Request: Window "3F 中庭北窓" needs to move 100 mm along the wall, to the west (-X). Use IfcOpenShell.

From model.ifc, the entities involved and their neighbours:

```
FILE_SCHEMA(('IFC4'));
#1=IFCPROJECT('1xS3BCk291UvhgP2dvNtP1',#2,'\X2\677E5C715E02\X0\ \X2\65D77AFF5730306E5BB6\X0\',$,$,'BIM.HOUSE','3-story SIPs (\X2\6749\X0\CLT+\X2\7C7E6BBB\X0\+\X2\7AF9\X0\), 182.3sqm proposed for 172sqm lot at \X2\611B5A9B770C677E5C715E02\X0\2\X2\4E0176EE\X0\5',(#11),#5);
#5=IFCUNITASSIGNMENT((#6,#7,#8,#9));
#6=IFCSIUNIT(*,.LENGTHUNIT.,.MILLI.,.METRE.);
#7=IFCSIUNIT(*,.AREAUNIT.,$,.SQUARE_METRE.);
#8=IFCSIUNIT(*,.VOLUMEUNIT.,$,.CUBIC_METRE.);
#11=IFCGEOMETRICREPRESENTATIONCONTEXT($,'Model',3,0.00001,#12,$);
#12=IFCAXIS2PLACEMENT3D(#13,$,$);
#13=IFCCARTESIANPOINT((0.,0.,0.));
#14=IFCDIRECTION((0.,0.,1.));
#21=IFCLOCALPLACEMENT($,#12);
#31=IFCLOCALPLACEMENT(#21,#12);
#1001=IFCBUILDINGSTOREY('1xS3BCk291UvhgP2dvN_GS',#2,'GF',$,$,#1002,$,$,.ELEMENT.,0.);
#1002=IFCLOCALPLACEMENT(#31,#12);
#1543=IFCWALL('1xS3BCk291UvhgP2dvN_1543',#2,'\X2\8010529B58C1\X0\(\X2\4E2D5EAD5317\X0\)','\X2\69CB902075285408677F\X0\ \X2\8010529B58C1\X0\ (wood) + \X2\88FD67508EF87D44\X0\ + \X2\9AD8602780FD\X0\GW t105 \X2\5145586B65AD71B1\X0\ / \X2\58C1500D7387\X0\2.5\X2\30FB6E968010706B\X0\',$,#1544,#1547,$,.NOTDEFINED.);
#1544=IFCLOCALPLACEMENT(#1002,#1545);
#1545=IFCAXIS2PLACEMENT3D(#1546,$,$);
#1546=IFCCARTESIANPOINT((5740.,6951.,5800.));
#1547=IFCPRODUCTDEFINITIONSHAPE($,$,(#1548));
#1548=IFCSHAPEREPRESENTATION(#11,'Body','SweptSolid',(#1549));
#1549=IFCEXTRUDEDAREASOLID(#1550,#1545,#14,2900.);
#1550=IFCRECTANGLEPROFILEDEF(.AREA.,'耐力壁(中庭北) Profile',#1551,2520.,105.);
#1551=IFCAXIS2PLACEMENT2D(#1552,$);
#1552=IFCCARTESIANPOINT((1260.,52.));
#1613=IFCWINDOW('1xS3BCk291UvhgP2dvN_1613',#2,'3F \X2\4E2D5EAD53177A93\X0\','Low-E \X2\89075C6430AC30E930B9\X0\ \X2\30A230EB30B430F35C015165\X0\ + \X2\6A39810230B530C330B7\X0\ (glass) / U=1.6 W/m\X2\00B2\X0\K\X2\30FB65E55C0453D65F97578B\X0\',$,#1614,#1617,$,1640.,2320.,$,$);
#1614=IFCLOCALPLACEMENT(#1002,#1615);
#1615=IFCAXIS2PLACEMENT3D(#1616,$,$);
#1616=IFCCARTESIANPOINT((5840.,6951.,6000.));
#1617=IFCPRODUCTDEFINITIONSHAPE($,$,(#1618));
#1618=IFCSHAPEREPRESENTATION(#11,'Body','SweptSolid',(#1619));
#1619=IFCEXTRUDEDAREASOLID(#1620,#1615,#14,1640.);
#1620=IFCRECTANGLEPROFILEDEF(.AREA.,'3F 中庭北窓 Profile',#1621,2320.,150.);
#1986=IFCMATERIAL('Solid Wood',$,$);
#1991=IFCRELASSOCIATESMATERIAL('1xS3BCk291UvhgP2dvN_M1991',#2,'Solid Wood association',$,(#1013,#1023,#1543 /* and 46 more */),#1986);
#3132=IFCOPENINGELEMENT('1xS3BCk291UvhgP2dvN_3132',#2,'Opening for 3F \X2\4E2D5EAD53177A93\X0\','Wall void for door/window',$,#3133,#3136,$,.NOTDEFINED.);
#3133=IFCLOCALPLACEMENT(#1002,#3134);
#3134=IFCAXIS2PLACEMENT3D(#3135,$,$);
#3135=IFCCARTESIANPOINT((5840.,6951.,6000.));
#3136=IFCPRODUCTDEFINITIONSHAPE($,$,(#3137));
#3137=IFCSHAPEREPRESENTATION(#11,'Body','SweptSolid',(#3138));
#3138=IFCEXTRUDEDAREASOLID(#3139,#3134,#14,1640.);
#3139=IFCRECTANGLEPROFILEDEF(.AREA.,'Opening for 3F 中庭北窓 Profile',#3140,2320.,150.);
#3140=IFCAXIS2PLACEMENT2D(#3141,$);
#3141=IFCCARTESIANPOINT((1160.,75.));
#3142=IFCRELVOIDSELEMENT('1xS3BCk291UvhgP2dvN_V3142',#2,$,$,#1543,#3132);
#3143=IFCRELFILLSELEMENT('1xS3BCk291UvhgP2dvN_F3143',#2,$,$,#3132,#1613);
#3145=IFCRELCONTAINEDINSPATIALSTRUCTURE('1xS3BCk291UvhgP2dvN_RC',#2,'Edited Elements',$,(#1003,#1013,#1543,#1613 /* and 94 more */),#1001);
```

```python
import ifcopenshell
import ifcopenshell.api.geometry
import ifcopenshell.util.placement
import ifcopenshell.util.unit

model = ifcopenshell.open("model.ifc")
unit_scale = ifcopenshell.util.unit.calculate_unit_scale(model)

window = model.by_guid("1xS3BCk291UvhgP2dvN_1613")
opening = window.FillsVoids[0].RelatingOpeningElement
wall = opening.VoidsElements[0].RelatingBuildingElement

wall_matrix = ifcopenshell.util.placement.get_local_placement(wall.ObjectPlacement)
shift = wall_matrix[:3, 0] * -0.1 / unit_scale
before = ifcopenshell.util.placement.get_local_placement(window.ObjectPlacement)[:3, 3].copy()

# The window is not placed relative to its opening, so move both.
for product in (opening, window):
    matrix = ifcopenshell.util.placement.get_local_placement(product.ObjectPlacement)
    matrix[:3, 3] += shift
    ifcopenshell.api.geometry.edit_object_placement(model, product=product, matrix=matrix, is_si=False)

after = ifcopenshell.util.placement.get_local_placement(window.ObjectPlacement)[:3, 3]
print("window moved by", (after - before).round(3) + 0.0)

model.write("model_updated.ifc")
```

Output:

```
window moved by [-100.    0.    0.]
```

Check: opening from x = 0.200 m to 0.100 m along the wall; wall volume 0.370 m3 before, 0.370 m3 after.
